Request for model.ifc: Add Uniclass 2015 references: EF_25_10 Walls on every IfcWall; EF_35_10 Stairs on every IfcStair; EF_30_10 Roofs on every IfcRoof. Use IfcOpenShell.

First a look at what the model holds.

```python
import ifcopenshell

model = ifcopenshell.open("model.ifc")
print(model.schema)
print("classifications:", [c.Name for c in model.by_type("IfcClassification")])
for ifc_class in ("IfcDoor", "IfcRoof", "IfcStair", "IfcWall", "IfcWindow"):
    print(ifc_class, len(model.by_type(ifc_class)))
```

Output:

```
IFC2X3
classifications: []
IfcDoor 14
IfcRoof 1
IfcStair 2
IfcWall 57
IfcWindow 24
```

```python
import ifcopenshell
import ifcopenshell.api.classification

model = ifcopenshell.open("model.ifc")

# IFC2X3 requires Source and Edition and has no link from the project to the system.
system = model.create_entity("IfcClassification", Source="NBS", Edition="2015", Name="Uniclass 2015")

codes = {
    "IfcWall": ("EF_25_10", "Walls"),
    "IfcStair": ("EF_35_10", "Stairs"),
    "IfcRoof": ("EF_30_10", "Roofs"),
}
for ifc_class, (code, name) in codes.items():
    products = model.by_type(ifc_class)
    ifcopenshell.api.classification.add_reference(
        model, products=products, classification=system, identification=code, name=name
    )
    print(code, len(products))

model.write("model_rev.ifc")
```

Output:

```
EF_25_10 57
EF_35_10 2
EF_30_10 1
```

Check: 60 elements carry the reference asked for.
